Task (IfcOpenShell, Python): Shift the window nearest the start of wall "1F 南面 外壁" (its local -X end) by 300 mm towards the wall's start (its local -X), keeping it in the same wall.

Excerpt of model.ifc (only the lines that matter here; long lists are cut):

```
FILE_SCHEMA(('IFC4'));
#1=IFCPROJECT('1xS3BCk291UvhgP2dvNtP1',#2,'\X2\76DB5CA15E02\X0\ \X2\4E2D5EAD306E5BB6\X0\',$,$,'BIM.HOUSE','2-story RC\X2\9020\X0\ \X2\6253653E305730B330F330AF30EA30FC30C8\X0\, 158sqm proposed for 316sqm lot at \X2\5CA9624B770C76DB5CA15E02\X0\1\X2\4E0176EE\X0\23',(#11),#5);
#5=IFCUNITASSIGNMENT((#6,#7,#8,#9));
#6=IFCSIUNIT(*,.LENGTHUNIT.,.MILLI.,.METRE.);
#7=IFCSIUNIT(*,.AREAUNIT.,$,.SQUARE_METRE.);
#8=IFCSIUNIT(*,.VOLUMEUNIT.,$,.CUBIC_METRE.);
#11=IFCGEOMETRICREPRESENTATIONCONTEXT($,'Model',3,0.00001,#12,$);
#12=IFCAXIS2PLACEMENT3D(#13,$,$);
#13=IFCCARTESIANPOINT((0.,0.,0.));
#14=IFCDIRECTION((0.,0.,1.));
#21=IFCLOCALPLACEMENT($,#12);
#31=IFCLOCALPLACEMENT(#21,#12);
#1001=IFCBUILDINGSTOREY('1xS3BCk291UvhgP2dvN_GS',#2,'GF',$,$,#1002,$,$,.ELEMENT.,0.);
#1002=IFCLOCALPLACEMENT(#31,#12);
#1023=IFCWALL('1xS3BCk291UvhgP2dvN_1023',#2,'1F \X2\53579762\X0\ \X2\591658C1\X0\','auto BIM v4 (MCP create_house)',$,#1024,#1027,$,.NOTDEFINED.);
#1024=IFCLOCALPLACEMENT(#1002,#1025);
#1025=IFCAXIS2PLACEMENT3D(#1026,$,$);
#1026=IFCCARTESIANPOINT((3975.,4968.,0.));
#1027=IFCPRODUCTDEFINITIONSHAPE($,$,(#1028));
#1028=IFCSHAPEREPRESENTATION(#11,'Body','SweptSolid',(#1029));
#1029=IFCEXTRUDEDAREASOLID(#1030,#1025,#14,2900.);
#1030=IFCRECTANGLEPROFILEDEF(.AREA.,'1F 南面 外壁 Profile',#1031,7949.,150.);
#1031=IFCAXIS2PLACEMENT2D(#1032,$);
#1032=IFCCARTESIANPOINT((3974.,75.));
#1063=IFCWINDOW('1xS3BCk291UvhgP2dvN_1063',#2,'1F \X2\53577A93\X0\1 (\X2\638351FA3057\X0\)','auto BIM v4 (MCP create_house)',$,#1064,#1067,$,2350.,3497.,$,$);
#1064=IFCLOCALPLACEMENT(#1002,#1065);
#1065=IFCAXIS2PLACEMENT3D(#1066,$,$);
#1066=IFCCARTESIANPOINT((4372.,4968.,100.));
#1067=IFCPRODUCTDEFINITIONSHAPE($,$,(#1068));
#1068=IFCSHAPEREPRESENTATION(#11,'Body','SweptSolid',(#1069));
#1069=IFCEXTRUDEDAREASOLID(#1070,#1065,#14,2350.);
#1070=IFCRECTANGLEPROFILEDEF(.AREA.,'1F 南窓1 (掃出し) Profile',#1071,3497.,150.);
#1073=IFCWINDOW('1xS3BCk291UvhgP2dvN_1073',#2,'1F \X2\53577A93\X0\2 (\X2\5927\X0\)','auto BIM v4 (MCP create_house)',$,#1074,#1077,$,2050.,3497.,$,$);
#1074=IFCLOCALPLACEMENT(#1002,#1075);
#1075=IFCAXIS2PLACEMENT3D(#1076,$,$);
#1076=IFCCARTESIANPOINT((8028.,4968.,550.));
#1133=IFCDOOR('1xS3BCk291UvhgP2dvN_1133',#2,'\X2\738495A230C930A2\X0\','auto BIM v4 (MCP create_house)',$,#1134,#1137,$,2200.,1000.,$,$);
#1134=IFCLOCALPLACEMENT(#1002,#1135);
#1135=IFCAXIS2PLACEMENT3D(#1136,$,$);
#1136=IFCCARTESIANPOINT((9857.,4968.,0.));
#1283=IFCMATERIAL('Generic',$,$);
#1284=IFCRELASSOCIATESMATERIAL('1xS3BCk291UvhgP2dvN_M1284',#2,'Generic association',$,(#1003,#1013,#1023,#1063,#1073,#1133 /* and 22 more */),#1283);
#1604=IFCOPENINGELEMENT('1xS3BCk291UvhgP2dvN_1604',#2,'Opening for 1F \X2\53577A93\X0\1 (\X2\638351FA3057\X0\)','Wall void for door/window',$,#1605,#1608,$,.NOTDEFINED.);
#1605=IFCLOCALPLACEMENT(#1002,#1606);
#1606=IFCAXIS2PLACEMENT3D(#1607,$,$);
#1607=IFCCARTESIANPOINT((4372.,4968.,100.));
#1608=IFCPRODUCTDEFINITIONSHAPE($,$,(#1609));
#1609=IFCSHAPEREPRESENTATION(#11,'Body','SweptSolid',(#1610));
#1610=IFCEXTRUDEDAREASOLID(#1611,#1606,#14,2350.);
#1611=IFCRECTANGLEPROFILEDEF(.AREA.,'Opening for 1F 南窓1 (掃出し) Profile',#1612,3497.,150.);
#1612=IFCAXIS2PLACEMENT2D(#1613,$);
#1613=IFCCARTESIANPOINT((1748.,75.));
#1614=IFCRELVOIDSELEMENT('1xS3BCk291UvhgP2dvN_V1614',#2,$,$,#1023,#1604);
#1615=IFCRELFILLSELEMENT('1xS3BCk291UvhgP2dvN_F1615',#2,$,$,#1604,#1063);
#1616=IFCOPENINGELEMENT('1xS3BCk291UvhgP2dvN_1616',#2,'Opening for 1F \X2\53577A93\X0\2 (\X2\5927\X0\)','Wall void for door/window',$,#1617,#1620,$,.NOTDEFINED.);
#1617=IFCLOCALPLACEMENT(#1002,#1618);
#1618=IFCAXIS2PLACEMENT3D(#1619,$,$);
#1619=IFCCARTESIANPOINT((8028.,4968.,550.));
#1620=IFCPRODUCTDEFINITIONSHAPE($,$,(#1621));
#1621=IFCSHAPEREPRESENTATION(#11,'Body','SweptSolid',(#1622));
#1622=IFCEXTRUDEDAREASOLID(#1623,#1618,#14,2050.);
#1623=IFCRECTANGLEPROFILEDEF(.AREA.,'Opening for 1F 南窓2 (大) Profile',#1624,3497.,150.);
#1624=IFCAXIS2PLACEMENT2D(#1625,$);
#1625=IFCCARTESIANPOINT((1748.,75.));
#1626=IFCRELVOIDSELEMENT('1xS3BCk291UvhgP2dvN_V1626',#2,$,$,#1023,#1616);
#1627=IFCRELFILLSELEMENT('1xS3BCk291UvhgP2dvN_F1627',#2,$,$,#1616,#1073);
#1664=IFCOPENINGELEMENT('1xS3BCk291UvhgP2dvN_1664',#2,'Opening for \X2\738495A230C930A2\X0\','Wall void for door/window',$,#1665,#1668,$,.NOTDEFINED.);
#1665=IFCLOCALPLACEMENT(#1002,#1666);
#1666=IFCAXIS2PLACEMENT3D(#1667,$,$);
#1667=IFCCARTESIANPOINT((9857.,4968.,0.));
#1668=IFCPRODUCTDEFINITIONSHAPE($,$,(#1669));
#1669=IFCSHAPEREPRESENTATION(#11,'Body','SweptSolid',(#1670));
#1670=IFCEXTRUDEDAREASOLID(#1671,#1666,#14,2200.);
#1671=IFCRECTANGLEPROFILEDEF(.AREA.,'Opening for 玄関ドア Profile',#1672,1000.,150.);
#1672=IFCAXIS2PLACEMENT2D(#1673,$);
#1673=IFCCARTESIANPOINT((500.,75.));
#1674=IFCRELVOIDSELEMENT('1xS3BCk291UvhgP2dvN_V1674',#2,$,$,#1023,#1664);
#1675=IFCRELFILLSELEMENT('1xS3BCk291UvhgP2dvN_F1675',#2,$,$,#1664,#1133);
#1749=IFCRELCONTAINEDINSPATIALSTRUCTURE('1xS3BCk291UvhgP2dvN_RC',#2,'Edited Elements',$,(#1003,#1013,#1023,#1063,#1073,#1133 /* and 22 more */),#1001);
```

```python
import ifcopenshell
import ifcopenshell.api.geometry
import ifcopenshell.util.placement
import ifcopenshell.util.unit

model = ifcopenshell.open("model.ifc")
unit_scale = ifcopenshell.util.unit.calculate_unit_scale(model)

window = model.by_guid("1xS3BCk291UvhgP2dvN_1063")
opening = window.FillsVoids[0].RelatingOpeningElement
wall = opening.VoidsElements[0].RelatingBuildingElement

wall_matrix = ifcopenshell.util.placement.get_local_placement(wall.ObjectPlacement)
shift = wall_matrix[:3, 0] * -0.3 / unit_scale
before = ifcopenshell.util.placement.get_local_placement(window.ObjectPlacement)[:3, 3].copy()

# The window is not placed relative to its opening, so move both.
for product in (opening, window):
    matrix = ifcopenshell.util.placement.get_local_placement(product.ObjectPlacement)
    matrix[:3, 3] += shift
    ifcopenshell.api.geometry.edit_object_placement(model, product=product, matrix=matrix, is_si=False)

after = ifcopenshell.util.placement.get_local_placement(window.ObjectPlacement)[:3, 3]
print("window moved by", (after - before).round(3) + 0.0)

model.write("model_updated.ifc")
```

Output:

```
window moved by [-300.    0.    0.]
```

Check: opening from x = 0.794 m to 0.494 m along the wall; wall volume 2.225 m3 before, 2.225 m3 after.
